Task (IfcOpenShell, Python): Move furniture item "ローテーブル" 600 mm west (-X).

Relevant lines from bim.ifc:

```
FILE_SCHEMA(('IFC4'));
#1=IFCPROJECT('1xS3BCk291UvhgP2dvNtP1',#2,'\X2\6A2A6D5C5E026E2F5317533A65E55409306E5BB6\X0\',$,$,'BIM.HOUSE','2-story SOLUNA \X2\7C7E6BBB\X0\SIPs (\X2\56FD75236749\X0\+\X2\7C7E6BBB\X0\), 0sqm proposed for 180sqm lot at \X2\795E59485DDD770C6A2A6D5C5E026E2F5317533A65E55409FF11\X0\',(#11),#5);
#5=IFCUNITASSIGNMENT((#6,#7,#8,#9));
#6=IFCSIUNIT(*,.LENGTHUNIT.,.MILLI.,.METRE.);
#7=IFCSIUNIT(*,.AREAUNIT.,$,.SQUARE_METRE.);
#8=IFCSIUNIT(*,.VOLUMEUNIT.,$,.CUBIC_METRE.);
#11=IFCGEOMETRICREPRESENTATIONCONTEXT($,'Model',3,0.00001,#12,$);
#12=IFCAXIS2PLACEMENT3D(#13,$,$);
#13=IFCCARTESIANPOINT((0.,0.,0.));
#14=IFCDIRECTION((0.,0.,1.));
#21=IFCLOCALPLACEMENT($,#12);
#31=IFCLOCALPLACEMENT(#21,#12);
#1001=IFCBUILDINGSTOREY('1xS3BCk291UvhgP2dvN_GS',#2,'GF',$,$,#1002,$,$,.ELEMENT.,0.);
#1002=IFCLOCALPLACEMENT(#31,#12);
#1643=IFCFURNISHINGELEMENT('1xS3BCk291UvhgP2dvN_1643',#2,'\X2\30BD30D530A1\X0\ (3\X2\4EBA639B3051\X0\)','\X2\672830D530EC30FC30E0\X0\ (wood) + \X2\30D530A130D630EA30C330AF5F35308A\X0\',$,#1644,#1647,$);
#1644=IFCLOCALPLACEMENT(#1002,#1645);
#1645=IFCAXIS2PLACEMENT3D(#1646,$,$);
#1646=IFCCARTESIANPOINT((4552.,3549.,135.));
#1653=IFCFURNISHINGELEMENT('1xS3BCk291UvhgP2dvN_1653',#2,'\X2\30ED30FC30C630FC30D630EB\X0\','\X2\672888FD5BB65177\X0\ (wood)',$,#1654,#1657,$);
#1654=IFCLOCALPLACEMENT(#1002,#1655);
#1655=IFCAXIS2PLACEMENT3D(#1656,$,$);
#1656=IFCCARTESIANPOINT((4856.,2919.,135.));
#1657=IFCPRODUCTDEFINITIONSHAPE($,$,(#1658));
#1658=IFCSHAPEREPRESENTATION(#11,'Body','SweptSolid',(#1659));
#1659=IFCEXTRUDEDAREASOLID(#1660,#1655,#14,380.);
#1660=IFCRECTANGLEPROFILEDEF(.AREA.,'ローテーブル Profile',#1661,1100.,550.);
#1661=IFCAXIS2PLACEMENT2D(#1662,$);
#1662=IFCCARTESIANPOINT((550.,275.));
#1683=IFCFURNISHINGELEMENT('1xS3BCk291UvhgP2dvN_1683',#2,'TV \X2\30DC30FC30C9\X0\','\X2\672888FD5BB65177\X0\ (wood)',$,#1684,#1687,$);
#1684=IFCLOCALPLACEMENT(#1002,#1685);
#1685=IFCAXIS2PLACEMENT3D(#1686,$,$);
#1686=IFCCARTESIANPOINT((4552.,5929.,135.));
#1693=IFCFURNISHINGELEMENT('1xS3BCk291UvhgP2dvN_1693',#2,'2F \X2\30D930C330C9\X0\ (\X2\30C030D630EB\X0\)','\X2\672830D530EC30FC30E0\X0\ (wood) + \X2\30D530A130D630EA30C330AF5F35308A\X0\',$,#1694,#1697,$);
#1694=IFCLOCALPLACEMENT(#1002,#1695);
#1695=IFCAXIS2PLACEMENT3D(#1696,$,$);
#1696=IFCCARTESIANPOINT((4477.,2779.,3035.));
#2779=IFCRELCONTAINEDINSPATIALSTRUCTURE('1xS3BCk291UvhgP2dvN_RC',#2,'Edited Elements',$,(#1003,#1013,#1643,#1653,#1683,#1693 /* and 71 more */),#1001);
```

```python
import ifcopenshell
import ifcopenshell.api.geometry
import ifcopenshell.util.placement

model = ifcopenshell.open("bim.ifc")

item = model.by_id(1653)
matrix = ifcopenshell.util.placement.get_local_placement(item.ObjectPlacement)
matrix[0, 3] -= 600.0
ifcopenshell.api.geometry.edit_object_placement(model, product=item, matrix=matrix, is_si=False)

print(ifcopenshell.util.placement.get_local_placement(item.ObjectPlacement).round(3) + 0.0)

model.write("bim_edited.ifc")
```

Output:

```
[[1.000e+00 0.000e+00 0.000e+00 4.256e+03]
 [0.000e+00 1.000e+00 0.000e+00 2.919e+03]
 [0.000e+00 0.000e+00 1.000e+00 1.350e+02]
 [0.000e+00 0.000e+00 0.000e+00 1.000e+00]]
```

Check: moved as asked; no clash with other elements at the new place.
